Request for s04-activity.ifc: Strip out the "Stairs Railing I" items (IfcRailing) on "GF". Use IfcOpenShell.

First a look at what the model holds.

```python
import ifcopenshell
import ifcopenshell.util.element

model = ifcopenshell.open("s04-activity.ifc")
print(model.schema)
storey = next(s for s in model.by_type("IfcBuildingStorey") if s.Name == "GF")
railings = [e for e in ifcopenshell.util.element.get_decomposition(storey) if e.is_a("IfcRailing")]
seen = {}
for e in railings:
    element_type = ifcopenshell.util.element.get_type(e)
    name = element_type.Name if element_type not in (None, e) else None
    seen[name] = seen.get(name, 0) + 1
for name, count in sorted(seen.items(), key=str):
    print(count, "x", name)
```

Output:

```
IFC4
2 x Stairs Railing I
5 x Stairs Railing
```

```python
import ifcopenshell
import ifcopenshell.api.root
import ifcopenshell.util.element

model = ifcopenshell.open("s04-activity.ifc")

storey = next(s for s in model.by_type("IfcBuildingStorey") if s.Name == "GF")
railings = [e for e in ifcopenshell.util.element.get_decomposition(storey) if e.is_a("IfcRailing")]
targets = [e for e in railings if (t := ifcopenshell.util.element.get_type(e)) not in (None, e) and t.Name == "Stairs Railing I"]

for e in targets:
    ifcopenshell.api.root.remove_product(model, product=e)
print(len(targets), "removed")

model.write("s04-activity-out.ifc")
```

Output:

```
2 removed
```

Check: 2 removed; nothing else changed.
